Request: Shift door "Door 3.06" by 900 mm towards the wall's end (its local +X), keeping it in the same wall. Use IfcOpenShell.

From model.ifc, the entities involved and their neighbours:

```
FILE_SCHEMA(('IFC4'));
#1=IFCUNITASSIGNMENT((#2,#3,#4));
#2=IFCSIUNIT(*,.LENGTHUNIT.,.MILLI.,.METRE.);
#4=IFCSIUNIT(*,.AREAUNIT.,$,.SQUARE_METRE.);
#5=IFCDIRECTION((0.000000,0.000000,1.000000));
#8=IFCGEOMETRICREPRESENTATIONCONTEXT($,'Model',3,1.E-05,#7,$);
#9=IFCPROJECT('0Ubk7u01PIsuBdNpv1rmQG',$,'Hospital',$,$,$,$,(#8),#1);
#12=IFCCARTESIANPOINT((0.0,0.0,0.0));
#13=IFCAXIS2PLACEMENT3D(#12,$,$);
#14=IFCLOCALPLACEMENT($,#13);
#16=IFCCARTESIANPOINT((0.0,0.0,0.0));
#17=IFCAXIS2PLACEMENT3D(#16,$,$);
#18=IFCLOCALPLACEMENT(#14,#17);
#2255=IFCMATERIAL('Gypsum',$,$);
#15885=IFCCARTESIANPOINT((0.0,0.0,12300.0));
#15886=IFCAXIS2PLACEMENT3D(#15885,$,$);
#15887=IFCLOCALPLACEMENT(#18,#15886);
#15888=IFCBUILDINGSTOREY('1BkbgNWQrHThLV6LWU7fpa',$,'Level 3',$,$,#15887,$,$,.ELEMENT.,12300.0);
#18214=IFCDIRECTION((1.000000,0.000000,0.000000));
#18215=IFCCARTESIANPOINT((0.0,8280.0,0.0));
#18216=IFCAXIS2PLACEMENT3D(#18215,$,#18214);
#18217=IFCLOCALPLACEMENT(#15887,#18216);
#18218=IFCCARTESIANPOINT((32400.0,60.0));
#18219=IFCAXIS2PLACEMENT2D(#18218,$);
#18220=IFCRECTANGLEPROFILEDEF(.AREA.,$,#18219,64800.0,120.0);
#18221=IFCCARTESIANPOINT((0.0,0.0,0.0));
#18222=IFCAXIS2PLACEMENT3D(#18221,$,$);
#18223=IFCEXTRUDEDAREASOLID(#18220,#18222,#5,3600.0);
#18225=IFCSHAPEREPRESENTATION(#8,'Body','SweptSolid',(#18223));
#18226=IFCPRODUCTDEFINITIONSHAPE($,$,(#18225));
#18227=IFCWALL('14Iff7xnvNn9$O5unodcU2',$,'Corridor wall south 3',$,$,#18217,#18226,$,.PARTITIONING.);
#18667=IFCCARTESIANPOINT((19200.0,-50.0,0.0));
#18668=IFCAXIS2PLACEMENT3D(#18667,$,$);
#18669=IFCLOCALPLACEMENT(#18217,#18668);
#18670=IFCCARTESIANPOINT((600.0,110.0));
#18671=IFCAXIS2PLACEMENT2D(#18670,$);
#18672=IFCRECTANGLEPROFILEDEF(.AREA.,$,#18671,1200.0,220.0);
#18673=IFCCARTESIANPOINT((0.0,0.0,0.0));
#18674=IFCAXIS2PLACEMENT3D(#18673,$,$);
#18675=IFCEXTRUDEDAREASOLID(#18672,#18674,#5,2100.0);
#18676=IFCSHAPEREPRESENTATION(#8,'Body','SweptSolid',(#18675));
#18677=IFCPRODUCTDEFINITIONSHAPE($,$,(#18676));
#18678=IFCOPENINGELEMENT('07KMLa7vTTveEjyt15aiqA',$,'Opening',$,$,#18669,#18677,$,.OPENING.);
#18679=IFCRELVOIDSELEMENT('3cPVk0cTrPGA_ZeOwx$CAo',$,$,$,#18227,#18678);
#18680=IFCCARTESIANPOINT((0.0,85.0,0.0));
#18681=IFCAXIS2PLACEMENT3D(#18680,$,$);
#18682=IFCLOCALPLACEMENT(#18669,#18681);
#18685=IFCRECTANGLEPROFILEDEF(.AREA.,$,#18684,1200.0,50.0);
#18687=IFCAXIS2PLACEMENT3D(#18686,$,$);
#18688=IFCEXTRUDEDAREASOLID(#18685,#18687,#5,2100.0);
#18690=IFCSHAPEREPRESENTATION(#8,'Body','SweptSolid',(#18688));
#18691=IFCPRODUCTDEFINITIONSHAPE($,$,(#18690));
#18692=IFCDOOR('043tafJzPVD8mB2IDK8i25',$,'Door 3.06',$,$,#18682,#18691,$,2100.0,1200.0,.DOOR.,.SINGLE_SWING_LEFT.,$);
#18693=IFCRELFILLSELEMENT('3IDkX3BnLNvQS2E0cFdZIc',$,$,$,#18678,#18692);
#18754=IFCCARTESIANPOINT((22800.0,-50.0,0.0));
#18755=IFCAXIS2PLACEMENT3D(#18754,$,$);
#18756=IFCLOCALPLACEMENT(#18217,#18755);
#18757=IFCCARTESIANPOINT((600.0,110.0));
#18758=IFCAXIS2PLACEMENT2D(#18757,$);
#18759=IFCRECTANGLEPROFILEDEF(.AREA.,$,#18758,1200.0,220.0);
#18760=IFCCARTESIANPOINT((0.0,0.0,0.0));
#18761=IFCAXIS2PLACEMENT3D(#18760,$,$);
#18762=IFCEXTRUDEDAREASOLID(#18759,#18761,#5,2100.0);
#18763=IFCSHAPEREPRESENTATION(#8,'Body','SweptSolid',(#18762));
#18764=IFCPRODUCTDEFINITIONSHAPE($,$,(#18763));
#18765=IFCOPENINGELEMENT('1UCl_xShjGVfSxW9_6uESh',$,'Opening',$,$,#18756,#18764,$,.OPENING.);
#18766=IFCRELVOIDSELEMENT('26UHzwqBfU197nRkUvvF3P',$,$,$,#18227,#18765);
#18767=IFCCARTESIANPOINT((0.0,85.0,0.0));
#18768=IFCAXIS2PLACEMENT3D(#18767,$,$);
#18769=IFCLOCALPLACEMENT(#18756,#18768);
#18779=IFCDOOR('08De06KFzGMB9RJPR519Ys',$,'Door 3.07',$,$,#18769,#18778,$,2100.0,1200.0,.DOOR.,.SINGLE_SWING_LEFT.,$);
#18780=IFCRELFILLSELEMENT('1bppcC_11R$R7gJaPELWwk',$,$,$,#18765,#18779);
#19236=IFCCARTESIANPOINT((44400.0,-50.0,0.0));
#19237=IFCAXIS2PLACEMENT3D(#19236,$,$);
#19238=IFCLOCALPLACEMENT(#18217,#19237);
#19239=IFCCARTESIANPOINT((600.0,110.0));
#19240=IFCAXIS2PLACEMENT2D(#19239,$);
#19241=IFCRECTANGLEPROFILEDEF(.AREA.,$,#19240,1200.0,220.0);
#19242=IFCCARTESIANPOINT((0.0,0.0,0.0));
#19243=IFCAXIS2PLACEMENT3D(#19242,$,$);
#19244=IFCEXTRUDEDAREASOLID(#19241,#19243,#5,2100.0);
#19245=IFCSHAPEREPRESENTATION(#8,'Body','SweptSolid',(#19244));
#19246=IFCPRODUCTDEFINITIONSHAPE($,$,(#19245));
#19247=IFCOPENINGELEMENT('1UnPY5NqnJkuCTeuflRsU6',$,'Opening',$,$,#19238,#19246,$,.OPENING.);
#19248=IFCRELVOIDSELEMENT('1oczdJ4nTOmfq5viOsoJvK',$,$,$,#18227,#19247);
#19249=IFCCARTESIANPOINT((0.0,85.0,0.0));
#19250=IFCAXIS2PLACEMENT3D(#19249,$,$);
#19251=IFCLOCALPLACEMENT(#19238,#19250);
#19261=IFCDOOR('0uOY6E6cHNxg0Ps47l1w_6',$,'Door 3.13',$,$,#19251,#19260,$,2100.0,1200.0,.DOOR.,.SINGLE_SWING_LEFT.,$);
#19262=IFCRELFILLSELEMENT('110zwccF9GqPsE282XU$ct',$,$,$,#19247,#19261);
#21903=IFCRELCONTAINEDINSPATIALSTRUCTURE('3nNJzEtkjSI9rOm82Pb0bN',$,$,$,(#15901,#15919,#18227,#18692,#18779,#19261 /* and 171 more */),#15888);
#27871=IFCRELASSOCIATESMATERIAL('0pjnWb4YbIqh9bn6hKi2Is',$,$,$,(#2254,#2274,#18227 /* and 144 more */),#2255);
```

```python
import ifcopenshell
import ifcopenshell.api.geometry
import ifcopenshell.util.placement
import ifcopenshell.util.unit

model = ifcopenshell.open("model.ifc")
unit_scale = ifcopenshell.util.unit.calculate_unit_scale(model)

door = model.by_guid("043tafJzPVD8mB2IDK8i25")
opening = door.FillsVoids[0].RelatingOpeningElement
wall = opening.VoidsElements[0].RelatingBuildingElement

wall_matrix = ifcopenshell.util.placement.get_local_placement(wall.ObjectPlacement)
shift = wall_matrix[:3, 0] * 0.9 / unit_scale
before = ifcopenshell.util.placement.get_local_placement(door.ObjectPlacement)[:3, 3].copy()

# The door is placed relative to its opening, so it follows when the opening moves.
matrix = ifcopenshell.util.placement.get_local_placement(opening.ObjectPlacement)
matrix[:3, 3] += shift
ifcopenshell.api.geometry.edit_object_placement(
    model, product=opening, matrix=matrix, is_si=False, should_transform_children=True
)

after = ifcopenshell.util.placement.get_local_placement(door.ObjectPlacement)[:3, 3]
print("door moved by", (after - before).round(3) + 0.0)

model.write("model_updated.ifc")
```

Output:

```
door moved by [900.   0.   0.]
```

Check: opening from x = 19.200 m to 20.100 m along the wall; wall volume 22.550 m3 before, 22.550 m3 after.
